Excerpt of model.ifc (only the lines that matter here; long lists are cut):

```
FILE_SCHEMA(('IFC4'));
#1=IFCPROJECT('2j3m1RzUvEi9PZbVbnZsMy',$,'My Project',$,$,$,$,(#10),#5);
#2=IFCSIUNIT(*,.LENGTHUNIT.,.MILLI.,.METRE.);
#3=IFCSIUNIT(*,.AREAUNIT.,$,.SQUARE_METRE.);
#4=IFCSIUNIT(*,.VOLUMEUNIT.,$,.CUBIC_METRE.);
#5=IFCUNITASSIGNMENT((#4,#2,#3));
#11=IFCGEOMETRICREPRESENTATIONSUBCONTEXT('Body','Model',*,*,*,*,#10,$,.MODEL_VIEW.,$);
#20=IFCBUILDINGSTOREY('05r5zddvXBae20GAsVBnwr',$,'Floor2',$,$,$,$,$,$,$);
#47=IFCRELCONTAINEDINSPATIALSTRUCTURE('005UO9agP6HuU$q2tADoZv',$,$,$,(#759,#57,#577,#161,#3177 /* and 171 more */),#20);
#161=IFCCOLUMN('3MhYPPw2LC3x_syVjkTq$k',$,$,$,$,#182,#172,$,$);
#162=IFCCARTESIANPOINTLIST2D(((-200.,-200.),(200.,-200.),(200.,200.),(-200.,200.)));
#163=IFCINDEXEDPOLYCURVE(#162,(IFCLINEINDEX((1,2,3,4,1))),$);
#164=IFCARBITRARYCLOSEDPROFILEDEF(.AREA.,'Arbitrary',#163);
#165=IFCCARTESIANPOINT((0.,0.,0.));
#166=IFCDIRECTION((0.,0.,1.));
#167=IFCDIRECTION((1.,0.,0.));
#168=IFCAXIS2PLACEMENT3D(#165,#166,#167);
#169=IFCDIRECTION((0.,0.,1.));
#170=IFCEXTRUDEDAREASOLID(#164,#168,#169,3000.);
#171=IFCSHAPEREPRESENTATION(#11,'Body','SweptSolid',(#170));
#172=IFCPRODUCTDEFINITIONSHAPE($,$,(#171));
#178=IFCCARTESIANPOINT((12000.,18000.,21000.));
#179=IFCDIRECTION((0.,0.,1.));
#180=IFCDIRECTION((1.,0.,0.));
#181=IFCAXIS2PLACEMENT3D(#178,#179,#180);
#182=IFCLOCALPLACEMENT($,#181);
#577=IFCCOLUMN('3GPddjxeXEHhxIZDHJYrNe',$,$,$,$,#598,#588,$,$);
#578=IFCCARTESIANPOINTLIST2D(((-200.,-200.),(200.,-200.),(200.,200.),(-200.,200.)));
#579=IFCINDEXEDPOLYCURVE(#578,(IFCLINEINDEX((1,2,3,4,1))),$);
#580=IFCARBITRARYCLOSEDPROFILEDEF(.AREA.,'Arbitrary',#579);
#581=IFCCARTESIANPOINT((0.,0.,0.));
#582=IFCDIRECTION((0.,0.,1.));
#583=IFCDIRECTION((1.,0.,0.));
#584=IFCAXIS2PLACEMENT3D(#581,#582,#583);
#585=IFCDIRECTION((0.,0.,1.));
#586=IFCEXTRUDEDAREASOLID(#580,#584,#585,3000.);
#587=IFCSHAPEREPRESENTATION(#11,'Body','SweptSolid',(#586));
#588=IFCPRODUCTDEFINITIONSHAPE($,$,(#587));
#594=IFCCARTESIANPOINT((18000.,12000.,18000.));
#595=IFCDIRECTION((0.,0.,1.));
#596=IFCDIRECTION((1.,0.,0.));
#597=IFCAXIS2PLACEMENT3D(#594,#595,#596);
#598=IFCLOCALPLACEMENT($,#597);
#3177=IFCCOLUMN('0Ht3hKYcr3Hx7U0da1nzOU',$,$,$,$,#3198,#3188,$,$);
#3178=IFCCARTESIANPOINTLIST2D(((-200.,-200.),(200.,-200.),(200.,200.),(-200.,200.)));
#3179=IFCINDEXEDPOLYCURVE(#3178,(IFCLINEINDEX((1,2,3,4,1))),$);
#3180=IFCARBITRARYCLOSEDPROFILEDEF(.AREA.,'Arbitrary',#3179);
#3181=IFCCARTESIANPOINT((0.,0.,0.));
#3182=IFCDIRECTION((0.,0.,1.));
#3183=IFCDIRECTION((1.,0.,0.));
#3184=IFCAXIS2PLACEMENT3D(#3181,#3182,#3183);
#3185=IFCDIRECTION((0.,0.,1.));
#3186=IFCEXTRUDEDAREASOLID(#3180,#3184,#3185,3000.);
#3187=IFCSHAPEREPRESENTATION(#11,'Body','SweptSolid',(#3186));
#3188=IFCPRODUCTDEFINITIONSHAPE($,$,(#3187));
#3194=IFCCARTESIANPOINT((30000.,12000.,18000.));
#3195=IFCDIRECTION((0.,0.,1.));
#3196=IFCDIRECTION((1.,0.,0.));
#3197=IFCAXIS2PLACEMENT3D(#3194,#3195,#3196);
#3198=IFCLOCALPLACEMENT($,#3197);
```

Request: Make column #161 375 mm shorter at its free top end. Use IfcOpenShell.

```python
import ifcopenshell
import ifcopenshell.util.representation
import ifcopenshell.util.unit

model = ifcopenshell.open("model.ifc")
unit_scale = ifcopenshell.util.unit.calculate_unit_scale(model)

member = model.by_guid("3MhYPPw2LC3x_syVjkTq$k")
change = -0.375 / unit_scale

# The extrusion runs towards the end named, so only its depth changes.
body = ifcopenshell.util.representation.get_representation(member, "Model", "Body")
solid = body.Items[0]
old_length = solid.Depth
solid.Depth += change

print(f"length {old_length:g} -> {solid.Depth:g}")

model.write("model_edited.ifc")
```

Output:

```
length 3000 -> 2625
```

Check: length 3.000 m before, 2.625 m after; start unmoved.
